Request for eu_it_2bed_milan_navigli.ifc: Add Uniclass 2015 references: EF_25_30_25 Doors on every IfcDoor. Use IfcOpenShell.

First a look at what the model holds.

```python
import ifcopenshell

model = ifcopenshell.open("eu_it_2bed_milan_navigli.ifc")
print(model.schema)
print("classifications:", [c.Name for c in model.by_type("IfcClassification")])
for ifc_class in ("IfcDoor", "IfcRoof", "IfcStair", "IfcWall", "IfcWindow"):
    print(ifc_class, len(model.by_type(ifc_class)))
```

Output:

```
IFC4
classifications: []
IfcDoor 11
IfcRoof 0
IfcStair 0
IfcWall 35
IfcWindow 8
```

```python
import ifcopenshell
import ifcopenshell.api.classification

model = ifcopenshell.open("eu_it_2bed_milan_navigli.ifc")

system = ifcopenshell.api.classification.add_classification(model, classification="Uniclass 2015")

codes = {
    "IfcDoor": ("EF_25_30_25", "Doors"),
}
for ifc_class, (code, name) in codes.items():
    products = model.by_type(ifc_class)
    ifcopenshell.api.classification.add_reference(
        model, products=products, classification=system, identification=code, name=name
    )
    print(code, len(products))

model.write("eu_it_2bed_milan_navigli_v2.ifc")
```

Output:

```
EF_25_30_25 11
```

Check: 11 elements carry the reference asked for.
